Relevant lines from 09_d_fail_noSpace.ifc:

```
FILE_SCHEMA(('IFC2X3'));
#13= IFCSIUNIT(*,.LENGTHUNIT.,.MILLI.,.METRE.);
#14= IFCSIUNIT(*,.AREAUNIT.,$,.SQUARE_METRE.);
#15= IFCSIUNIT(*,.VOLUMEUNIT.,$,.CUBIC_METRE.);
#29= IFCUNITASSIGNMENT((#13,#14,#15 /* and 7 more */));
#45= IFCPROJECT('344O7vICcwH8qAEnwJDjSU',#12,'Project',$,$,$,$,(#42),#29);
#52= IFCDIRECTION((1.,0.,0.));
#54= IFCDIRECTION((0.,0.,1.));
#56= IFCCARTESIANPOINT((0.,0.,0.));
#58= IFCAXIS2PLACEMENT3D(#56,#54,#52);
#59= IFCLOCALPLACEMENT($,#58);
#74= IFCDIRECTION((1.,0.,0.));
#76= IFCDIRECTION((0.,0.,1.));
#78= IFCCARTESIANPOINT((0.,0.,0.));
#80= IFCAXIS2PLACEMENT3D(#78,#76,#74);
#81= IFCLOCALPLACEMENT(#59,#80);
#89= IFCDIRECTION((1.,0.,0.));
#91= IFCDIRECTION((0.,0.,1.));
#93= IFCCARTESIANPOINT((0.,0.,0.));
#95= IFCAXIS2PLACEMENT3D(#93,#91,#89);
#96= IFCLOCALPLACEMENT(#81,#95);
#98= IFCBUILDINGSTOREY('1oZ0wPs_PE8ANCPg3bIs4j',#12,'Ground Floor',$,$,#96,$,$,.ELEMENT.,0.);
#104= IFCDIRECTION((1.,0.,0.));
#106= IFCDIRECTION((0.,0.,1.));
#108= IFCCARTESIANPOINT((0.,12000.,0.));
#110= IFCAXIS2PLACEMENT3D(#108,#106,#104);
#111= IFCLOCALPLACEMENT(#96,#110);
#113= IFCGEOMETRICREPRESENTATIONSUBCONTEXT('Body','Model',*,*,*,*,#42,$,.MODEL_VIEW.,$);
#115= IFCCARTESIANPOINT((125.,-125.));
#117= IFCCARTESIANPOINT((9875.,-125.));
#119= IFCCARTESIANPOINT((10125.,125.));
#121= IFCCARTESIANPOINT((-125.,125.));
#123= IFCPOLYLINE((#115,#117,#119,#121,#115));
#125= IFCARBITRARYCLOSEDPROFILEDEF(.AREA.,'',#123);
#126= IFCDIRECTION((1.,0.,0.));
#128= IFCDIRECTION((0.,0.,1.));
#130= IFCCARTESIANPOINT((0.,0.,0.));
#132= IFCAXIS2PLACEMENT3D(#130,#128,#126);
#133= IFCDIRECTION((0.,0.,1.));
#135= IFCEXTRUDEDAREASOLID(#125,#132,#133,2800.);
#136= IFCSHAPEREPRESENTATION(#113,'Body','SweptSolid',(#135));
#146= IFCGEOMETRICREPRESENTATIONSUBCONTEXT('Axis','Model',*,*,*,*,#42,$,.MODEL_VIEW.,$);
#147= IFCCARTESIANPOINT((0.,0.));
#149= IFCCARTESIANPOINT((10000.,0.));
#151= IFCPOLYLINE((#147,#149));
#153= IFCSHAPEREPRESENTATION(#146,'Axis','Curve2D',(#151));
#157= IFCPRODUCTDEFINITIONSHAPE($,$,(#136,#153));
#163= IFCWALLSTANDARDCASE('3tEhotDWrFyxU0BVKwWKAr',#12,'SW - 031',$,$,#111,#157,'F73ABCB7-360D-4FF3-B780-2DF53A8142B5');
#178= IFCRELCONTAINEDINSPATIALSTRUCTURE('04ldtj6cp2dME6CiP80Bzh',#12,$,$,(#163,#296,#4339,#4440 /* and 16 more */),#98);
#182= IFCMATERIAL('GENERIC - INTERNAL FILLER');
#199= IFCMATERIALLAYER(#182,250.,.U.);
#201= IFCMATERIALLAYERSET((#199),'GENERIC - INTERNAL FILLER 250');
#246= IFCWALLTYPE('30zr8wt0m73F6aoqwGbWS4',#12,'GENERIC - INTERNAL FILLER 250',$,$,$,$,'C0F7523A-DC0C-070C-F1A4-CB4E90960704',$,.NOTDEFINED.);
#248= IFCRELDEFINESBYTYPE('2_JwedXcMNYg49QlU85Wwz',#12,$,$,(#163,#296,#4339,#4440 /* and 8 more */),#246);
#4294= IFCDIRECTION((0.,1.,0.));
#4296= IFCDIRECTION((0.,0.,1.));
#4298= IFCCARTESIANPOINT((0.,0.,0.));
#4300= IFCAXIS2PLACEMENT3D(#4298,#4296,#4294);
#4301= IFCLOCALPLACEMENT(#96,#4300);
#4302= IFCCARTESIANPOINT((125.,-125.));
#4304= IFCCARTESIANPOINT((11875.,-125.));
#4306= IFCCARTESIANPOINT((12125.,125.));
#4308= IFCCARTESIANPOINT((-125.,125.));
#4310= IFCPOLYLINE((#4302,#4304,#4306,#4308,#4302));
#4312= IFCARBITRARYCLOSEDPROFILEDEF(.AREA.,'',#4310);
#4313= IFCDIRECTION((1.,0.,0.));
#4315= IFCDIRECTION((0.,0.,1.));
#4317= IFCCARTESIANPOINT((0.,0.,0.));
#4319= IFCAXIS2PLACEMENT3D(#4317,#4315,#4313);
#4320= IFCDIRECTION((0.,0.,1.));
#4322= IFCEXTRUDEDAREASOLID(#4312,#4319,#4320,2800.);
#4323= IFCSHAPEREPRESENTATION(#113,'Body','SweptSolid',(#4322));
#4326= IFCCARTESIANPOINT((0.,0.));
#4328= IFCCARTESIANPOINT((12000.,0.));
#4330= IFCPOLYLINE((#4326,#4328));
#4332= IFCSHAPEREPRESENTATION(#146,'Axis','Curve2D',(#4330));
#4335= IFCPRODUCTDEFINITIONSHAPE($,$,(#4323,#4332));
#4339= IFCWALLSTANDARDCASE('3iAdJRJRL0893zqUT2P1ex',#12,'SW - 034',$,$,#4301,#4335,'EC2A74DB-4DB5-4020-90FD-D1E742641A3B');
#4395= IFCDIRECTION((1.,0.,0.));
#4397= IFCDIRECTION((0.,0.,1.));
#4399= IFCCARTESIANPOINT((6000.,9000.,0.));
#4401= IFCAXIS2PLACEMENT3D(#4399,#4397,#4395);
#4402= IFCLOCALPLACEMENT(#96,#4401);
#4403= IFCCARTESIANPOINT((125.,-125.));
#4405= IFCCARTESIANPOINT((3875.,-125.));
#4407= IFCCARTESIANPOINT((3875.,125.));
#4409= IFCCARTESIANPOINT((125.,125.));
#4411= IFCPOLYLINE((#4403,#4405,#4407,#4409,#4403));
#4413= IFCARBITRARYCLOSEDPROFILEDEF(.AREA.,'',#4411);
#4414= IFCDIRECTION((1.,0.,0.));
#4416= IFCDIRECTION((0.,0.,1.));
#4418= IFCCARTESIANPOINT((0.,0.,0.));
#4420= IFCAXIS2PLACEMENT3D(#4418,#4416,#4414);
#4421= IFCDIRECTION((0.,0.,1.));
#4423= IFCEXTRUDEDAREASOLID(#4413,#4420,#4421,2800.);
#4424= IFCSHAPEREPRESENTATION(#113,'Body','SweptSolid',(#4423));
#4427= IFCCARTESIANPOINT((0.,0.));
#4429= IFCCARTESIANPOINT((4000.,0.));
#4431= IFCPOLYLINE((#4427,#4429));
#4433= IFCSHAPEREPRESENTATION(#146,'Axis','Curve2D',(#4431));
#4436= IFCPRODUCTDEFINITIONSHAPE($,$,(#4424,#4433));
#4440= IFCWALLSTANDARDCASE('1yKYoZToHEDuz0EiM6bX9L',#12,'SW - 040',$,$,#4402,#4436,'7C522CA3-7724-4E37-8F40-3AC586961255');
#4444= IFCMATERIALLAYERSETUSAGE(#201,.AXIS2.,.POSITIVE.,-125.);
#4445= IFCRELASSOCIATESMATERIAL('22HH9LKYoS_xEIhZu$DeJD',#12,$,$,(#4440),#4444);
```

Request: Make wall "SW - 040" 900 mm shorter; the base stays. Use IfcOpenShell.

```python
import ifcopenshell
import ifcopenshell.geom
import ifcopenshell.util.representation
import ifcopenshell.util.shape
import ifcopenshell.util.unit

model = ifcopenshell.open("09_d_fail_noSpace.ifc")
unit_scale = ifcopenshell.util.unit.calculate_unit_scale(model)
settings = ifcopenshell.geom.settings()


def volume(element):
    """Net volume in cubic metres, openings subtracted."""
    shape = ifcopenshell.geom.create_shape(settings, element)
    return ifcopenshell.util.shape.get_volume(shape.geometry)


wall = model.by_id(4440)
before = volume(wall)

body = ifcopenshell.util.representation.get_representation(wall, "Model", "Body")
solid = body.Items[0]
old_height = solid.Depth
solid.Depth -= 0.9 / unit_scale
after = volume(wall)

print(f"height {old_height:g} -> {solid.Depth:g}, volume {before:.3f} -> {after:.3f} m3")

model.write("09_d_fail_noSpace_edited.ifc")
```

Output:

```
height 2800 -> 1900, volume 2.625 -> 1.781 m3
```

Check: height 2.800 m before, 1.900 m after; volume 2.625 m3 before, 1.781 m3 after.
